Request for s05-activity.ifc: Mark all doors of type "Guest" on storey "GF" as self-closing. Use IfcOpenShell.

First a look at what the model holds.

```python
import ifcopenshell
import ifcopenshell.util.element

model = ifcopenshell.open("s05-activity.ifc")
print(model.schema)
storey = next(s for s in model.by_type("IfcBuildingStorey") if s.Name == "GF")
doors = [e for e in ifcopenshell.util.element.get_decomposition(storey) if e.is_a("IfcDoor")]
seen = {}
for e in doors:
    element_type = ifcopenshell.util.element.get_type(e)
    key = (element_type.Name if element_type != e and element_type else None, ifcopenshell.util.element.get_pset(e, "Pset_DoorCommon", "SelfClosing"))
    seen[key] = seen.get(key, 0) + 1
for (name, value), count in sorted(seen.items(), key=str):
    print(count, "x", name, "|", value)
```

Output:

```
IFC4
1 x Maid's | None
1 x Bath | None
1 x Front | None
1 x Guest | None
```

```python
import ifcopenshell
import ifcopenshell.api.pset
import ifcopenshell.util.element

model = ifcopenshell.open("s05-activity.ifc")

storey = next(s for s in model.by_type("IfcBuildingStorey") if s.Name == "GF")
doors = [e for e in ifcopenshell.util.element.get_decomposition(storey) if e.is_a("IfcDoor")]

count = 0
for e in doors:
    element_type = ifcopenshell.util.element.get_type(e)
    if element_type in (None, e) or element_type.Name != "Guest":
        continue
    # add_pset returns the element's existing set when there is one.
    pset = ifcopenshell.api.pset.add_pset(model, product=e, name="Pset_DoorCommon")
    ifcopenshell.api.pset.edit_pset(model, pset=pset, properties={"SelfClosing": True})
    count += 1

print(count, "doors updated")

model.write("s05-activity-out.ifc")
```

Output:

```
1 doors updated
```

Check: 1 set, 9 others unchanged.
